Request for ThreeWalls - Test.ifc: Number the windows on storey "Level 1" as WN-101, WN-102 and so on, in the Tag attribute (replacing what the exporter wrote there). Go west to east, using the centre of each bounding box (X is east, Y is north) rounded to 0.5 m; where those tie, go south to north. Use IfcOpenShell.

First a look at what the model holds.

```python
import ifcopenshell
import ifcopenshell.util.element
import ifcopenshell.util.placement

model = ifcopenshell.open("ThreeWalls - Test.ifc")
print(model.schema)
storey = next(s for s in model.by_type("IfcBuildingStorey") if s.Name == "Level 1")
windows = [e for e in ifcopenshell.util.element.get_decomposition(storey) if e.is_a("IfcWindow")]
for e in sorted(windows, key=lambda e: e.id()):
    origin = ifcopenshell.util.placement.get_local_placement(e.ObjectPlacement)[:3, 3]
    print(e.id(), e.Tag, e.Name, origin.round(2) + 0.0, sep=" | ")
```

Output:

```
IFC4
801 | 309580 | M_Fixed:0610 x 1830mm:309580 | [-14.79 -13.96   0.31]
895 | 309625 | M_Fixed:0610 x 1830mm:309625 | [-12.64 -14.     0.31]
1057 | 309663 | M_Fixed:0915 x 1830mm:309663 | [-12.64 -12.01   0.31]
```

```python
import ifcopenshell
import ifcopenshell.geom
import ifcopenshell.util.element
import ifcopenshell.util.shape

model = ifcopenshell.open("ThreeWalls - Test.ifc")
settings = ifcopenshell.geom.settings()
settings.set("use-world-coords", True)


def centre(element):
    shape = ifcopenshell.geom.create_shape(settings, element)
    return ifcopenshell.util.shape.get_bbox_centroid(shape.geometry)


storey = next(s for s in model.by_type("IfcBuildingStorey") if s.Name == "Level 1")
windows = [e for e in ifcopenshell.util.element.get_decomposition(storey) if e.is_a("IfcWindow")]

# Insertion points can sit at a corner or the storey origin, so sort by the geometry (in metres).
centres = {e: centre(e) for e in windows}
windows.sort(key=lambda e: (round(centres[e][0] / 0.5), centres[e][1]))

for i, e in enumerate(windows, start=1):
    number = f"WN-1{i:02d}"
    e.Tag = number
    print(e.id(), number)

model.write("ThreeWalls - Test_updated.ifc")
```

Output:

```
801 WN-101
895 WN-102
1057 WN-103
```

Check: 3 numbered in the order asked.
